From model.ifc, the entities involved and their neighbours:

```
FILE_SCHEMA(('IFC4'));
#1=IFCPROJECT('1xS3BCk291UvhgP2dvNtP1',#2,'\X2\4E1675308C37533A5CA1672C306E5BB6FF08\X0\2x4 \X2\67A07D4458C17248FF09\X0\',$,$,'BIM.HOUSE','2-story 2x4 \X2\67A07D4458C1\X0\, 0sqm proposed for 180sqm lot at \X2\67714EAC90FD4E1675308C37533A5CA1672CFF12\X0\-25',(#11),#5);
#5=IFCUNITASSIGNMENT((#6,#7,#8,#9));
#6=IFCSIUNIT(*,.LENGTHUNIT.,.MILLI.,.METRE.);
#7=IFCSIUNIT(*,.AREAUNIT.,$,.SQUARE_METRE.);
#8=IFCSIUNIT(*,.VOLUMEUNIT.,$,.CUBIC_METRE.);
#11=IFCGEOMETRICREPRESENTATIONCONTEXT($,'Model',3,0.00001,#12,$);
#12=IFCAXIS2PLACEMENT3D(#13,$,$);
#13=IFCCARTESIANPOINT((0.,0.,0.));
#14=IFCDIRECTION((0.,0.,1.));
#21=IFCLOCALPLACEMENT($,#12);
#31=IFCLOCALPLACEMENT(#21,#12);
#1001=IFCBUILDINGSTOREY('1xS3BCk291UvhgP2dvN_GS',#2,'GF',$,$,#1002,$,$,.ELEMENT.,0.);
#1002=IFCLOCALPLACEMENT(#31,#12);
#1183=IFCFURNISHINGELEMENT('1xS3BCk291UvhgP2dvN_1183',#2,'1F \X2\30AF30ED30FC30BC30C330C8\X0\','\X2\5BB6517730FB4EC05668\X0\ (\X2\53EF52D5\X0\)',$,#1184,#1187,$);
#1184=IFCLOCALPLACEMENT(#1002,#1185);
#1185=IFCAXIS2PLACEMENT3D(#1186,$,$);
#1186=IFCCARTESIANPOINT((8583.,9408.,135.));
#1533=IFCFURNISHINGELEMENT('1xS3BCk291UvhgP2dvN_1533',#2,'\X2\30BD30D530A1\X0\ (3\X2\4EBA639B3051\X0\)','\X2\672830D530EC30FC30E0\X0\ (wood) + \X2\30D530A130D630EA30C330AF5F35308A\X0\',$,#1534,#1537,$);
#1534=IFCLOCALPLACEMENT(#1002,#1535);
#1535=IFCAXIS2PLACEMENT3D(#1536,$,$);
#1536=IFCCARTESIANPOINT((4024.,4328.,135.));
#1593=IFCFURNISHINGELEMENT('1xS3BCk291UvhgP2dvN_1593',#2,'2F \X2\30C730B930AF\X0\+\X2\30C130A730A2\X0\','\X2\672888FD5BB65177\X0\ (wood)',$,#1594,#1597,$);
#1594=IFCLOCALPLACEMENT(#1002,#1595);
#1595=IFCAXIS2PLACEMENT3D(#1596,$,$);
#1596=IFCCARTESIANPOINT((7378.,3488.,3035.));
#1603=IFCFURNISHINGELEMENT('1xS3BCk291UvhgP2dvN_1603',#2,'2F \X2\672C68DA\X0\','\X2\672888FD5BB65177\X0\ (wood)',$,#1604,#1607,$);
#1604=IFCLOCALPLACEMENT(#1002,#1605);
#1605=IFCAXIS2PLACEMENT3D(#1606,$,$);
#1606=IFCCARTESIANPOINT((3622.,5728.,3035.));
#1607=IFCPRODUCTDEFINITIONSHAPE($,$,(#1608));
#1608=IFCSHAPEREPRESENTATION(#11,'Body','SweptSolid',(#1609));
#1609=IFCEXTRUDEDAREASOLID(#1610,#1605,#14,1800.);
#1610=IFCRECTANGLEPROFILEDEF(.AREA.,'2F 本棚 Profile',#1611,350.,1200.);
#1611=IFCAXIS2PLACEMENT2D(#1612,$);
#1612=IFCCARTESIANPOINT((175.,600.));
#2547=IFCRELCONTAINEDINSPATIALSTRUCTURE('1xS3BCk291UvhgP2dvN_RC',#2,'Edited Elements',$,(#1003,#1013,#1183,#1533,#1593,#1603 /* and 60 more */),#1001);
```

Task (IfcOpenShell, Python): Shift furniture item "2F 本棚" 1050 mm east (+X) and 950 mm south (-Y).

```python
import ifcopenshell
import ifcopenshell.api.geometry
import ifcopenshell.util.placement
import ifcopenshell.util.unit

model = ifcopenshell.open("model.ifc")
unit_scale = ifcopenshell.util.unit.calculate_unit_scale(model)

item = model.by_guid("1xS3BCk291UvhgP2dvN_1603")
matrix = ifcopenshell.util.placement.get_local_placement(item.ObjectPlacement)
matrix[0, 3] += 1.05 / unit_scale
matrix[1, 3] -= 0.95 / unit_scale
ifcopenshell.api.geometry.edit_object_placement(model, product=item, matrix=matrix, is_si=False)

print(ifcopenshell.util.placement.get_local_placement(item.ObjectPlacement).round(3) + 0.0)

model.write("model_rev.ifc")
```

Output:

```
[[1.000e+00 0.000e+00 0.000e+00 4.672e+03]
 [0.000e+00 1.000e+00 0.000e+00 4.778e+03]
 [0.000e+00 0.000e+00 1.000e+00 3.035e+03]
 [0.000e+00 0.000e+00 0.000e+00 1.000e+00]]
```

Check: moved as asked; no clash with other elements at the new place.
